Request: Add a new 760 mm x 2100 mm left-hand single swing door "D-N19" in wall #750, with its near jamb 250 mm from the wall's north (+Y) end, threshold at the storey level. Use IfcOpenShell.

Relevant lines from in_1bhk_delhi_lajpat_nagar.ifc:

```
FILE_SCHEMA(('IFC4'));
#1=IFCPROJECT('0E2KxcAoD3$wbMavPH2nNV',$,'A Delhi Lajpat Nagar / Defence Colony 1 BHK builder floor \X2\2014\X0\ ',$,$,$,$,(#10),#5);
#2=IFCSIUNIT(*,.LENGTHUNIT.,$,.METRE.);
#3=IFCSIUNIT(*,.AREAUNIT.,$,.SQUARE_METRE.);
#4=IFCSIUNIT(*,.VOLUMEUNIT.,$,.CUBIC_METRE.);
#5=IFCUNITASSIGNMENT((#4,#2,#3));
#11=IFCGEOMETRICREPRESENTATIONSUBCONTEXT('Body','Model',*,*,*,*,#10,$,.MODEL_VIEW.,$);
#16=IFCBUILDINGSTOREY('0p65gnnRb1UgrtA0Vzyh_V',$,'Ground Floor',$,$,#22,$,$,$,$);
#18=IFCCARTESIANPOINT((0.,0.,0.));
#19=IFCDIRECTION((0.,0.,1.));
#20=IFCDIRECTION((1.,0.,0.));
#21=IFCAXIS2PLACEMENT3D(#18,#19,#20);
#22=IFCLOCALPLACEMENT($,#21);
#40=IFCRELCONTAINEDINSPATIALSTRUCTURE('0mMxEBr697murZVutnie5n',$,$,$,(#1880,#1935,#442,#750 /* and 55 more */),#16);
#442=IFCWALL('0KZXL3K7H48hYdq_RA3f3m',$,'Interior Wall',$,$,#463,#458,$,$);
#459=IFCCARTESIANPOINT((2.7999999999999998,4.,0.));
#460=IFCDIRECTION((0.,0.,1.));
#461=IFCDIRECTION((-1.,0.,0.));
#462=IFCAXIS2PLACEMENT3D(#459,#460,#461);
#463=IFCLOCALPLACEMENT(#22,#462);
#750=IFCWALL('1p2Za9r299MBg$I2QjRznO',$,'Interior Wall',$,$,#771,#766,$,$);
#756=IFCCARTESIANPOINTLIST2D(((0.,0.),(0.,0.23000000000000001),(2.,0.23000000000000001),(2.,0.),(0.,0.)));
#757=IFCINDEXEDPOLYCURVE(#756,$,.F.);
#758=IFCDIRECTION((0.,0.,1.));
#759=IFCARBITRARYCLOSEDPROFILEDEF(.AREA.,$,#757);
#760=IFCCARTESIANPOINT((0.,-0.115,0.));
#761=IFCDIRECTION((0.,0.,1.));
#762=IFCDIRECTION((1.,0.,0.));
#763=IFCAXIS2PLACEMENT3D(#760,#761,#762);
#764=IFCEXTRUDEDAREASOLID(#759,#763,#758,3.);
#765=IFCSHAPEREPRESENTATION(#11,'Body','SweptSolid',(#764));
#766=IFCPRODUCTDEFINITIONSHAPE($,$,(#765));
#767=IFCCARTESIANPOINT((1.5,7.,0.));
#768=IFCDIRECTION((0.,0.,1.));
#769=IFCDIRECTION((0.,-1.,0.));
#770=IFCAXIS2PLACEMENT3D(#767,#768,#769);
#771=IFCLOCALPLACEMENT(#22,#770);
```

```python
import numpy as np
import ifcopenshell
import ifcopenshell.api.feature
import ifcopenshell.api.geometry
import ifcopenshell.api.root
import ifcopenshell.api.spatial
import ifcopenshell.geom
import ifcopenshell.util.element
import ifcopenshell.util.placement
import ifcopenshell.util.representation
import ifcopenshell.util.shape
import ifcopenshell.util.unit

model = ifcopenshell.open("in_1bhk_delhi_lajpat_nagar.ifc")
unit_scale = ifcopenshell.util.unit.calculate_unit_scale(model)
settings = ifcopenshell.geom.settings()


def volume(element):
    """Net volume in cubic metres, openings subtracted."""
    shape = ifcopenshell.geom.create_shape(settings, element)
    return ifcopenshell.util.shape.get_volume(shape.geometry)


wall = model.by_guid("1p2Za9r299MBg$I2QjRznO")
storey = ifcopenshell.util.element.get_container(wall, ifc_class="IfcBuildingStorey")
context = ifcopenshell.util.representation.get_context(model, "Model", "Body", "MODEL_VIEW")
before = volume(wall)

width, height, from_end, sill = 0.76, 2.1, 0.25, 0.0  # metres

# The wall runs along its own X axis, and the end named is its -X end.
wall_shape = ifcopenshell.geom.create_shape(settings, wall)
x, y, z = ifcopenshell.util.shape.get_vertices(wall_shape.geometry).T
start = x.min() + from_end
face, thickness = float(y.min()), float(y.max() - y.min())
wall_matrix = ifcopenshell.util.placement.get_local_placement(wall.ObjectPlacement)
level = ifcopenshell.util.placement.get_local_placement(storey.ObjectPlacement)[2, 3]


def in_wall(x, y):
    """Placement at x, y metres in the wall's axes, at sill height."""
    matrix = wall_matrix.copy()
    matrix[:, 3] = wall_matrix @ np.array([x / unit_scale, y / unit_scale, 0.0, 1.0])
    matrix[2, 3] = level + sill / unit_scale
    return matrix


# Opening: a box that overshoots both wall faces by 50 mm.
opening = ifcopenshell.api.root.create_entity(model, ifc_class="IfcOpeningElement", predefined_type="OPENING")
box = ifcopenshell.api.geometry.add_wall_representation(
    model, context=context, length=width, height=height, thickness=thickness + 0.1
)
ifcopenshell.api.geometry.assign_representation(model, product=opening, representation=box)
ifcopenshell.api.geometry.edit_object_placement(model, product=opening, matrix=in_wall(start, face - 0.05), is_si=False)
ifcopenshell.api.feature.add_feature(model, feature=opening, element=wall)

door = ifcopenshell.api.root.create_entity(model, ifc_class="IfcDoor", name="D-N19", predefined_type="DOOR")
door.OverallWidth, door.OverallHeight = width / unit_scale, height / unit_scale
door.OperationType = "SINGLE_SWING_LEFT"
body = ifcopenshell.api.geometry.add_door_representation(
    model,
    context=context,
    overall_width=door.OverallWidth,
    overall_height=door.OverallHeight,
    operation_type="SINGLE_SWING_LEFT",
    lining_properties={"LiningDepth": thickness / unit_scale, "ThresholdDepth": thickness / unit_scale},
)
ifcopenshell.api.geometry.assign_representation(model, product=door, representation=body)
ifcopenshell.api.spatial.assign_container(model, products=[door], relating_structure=storey)
ifcopenshell.api.feature.add_filling(model, opening=opening, element=door)

# The lining spans the wall, so the door starts at the wall face.
ifcopenshell.api.geometry.edit_object_placement(model, product=door, matrix=in_wall(start, face), is_si=False)

after = volume(wall)

print(f"wall volume {before:.3f} -> {after:.3f} m3")

model.write("in_1bhk_delhi_lajpat_nagar-out.ifc")
```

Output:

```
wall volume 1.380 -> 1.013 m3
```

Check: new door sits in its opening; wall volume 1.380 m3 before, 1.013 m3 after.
